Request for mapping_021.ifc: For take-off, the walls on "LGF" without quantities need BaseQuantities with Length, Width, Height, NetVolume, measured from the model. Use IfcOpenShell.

First a look at what the model holds.

```python
import ifcopenshell
import ifcopenshell.util.element
import ifcopenshell.util.unit

model = ifcopenshell.open("mapping_021.ifc")
print(model.schema)
for unit_type in ("LENGTHUNIT", "AREAUNIT", "VOLUMEUNIT"):
    print(unit_type, ifcopenshell.util.unit.calculate_unit_scale(model, unit_type))
storey = next(s for s in model.by_type("IfcBuildingStorey") if s.Name == "LGF")
walls = [e for e in ifcopenshell.util.element.get_decomposition(storey) if e.is_a("IfcWall")]
for e in sorted(walls, key=lambda e: e.id()):
    print(e.id(), e.is_a(), e.Name, list(ifcopenshell.util.element.get_psets(e, qtos_only=True)), sep=" | ")
```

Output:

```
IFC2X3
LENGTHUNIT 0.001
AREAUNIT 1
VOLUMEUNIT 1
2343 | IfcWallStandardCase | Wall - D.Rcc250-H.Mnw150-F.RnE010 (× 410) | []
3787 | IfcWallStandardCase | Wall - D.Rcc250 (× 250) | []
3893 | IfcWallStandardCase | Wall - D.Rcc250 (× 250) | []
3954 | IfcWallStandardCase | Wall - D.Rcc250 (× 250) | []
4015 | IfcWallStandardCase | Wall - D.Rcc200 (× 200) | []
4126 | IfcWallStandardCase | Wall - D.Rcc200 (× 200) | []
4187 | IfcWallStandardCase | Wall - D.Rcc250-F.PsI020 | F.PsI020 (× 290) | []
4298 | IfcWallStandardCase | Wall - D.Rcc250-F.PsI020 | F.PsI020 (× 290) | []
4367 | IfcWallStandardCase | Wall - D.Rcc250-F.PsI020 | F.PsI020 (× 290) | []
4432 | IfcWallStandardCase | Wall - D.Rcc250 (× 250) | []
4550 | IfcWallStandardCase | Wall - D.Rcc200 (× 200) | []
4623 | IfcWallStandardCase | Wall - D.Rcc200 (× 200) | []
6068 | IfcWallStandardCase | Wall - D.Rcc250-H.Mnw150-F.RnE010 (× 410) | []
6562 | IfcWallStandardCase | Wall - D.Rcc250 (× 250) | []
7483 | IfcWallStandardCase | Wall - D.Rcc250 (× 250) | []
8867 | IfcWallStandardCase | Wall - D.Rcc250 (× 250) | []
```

```python
import ifcopenshell
import ifcopenshell.api.pset
import ifcopenshell.geom
import ifcopenshell.util.element
import ifcopenshell.util.shape
import ifcopenshell.util.unit

model = ifcopenshell.open("mapping_021.ifc")
unit_scale = ifcopenshell.util.unit.calculate_unit_scale(model)
volume_scale = ifcopenshell.util.unit.calculate_unit_scale(model, "VOLUMEUNIT")
settings = ifcopenshell.geom.settings()

storey = next(s for s in model.by_type("IfcBuildingStorey") if s.Name == "LGF")
walls = [e for e in ifcopenshell.util.element.get_decomposition(storey) if e.is_a("IfcWall")]

for e in sorted(walls, key=lambda e: e.id()):
    if ifcopenshell.util.element.get_psets(e, qtos_only=True, should_inherit=False):
        continue
    # Geometry comes back in metres, in the element's own axes.
    shape = ifcopenshell.geom.create_shape(settings, e)
    values = {
        "Length": ifcopenshell.util.shape.get_x(shape.geometry) / unit_scale,
        "Width": ifcopenshell.util.shape.get_y(shape.geometry) / unit_scale,
        "Height": ifcopenshell.util.shape.get_z(shape.geometry) / unit_scale,
        "NetVolume": ifcopenshell.util.shape.get_volume(shape.geometry) / volume_scale,
    }
    qto = ifcopenshell.api.pset.add_qto(model, product=e, name="BaseQuantities")
    ifcopenshell.api.pset.edit_qto(model, qto=qto, properties=values)
    print(e.id(), {k: round(v, 3) for k, v in values.items()})

model.write("mapping_021_rev.ifc")
```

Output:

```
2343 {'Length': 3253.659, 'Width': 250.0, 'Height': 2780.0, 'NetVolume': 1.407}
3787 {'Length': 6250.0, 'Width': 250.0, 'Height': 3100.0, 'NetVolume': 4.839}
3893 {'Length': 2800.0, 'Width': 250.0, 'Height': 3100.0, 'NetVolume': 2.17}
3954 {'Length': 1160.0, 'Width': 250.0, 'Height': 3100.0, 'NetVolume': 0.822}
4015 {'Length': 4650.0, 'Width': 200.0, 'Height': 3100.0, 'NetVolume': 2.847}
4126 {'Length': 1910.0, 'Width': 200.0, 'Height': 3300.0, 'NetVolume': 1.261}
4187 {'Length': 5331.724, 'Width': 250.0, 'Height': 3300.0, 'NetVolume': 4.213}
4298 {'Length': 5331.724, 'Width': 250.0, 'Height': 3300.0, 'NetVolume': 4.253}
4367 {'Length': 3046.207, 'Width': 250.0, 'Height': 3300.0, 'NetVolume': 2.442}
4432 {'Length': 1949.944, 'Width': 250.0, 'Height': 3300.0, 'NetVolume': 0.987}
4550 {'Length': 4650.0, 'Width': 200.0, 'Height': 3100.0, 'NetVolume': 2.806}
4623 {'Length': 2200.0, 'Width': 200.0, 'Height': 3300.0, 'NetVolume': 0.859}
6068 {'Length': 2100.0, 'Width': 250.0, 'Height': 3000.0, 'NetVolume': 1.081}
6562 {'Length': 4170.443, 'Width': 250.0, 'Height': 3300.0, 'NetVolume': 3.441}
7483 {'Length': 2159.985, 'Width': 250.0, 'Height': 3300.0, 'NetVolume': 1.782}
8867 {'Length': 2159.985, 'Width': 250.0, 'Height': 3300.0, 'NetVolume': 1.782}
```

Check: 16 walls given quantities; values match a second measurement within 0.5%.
